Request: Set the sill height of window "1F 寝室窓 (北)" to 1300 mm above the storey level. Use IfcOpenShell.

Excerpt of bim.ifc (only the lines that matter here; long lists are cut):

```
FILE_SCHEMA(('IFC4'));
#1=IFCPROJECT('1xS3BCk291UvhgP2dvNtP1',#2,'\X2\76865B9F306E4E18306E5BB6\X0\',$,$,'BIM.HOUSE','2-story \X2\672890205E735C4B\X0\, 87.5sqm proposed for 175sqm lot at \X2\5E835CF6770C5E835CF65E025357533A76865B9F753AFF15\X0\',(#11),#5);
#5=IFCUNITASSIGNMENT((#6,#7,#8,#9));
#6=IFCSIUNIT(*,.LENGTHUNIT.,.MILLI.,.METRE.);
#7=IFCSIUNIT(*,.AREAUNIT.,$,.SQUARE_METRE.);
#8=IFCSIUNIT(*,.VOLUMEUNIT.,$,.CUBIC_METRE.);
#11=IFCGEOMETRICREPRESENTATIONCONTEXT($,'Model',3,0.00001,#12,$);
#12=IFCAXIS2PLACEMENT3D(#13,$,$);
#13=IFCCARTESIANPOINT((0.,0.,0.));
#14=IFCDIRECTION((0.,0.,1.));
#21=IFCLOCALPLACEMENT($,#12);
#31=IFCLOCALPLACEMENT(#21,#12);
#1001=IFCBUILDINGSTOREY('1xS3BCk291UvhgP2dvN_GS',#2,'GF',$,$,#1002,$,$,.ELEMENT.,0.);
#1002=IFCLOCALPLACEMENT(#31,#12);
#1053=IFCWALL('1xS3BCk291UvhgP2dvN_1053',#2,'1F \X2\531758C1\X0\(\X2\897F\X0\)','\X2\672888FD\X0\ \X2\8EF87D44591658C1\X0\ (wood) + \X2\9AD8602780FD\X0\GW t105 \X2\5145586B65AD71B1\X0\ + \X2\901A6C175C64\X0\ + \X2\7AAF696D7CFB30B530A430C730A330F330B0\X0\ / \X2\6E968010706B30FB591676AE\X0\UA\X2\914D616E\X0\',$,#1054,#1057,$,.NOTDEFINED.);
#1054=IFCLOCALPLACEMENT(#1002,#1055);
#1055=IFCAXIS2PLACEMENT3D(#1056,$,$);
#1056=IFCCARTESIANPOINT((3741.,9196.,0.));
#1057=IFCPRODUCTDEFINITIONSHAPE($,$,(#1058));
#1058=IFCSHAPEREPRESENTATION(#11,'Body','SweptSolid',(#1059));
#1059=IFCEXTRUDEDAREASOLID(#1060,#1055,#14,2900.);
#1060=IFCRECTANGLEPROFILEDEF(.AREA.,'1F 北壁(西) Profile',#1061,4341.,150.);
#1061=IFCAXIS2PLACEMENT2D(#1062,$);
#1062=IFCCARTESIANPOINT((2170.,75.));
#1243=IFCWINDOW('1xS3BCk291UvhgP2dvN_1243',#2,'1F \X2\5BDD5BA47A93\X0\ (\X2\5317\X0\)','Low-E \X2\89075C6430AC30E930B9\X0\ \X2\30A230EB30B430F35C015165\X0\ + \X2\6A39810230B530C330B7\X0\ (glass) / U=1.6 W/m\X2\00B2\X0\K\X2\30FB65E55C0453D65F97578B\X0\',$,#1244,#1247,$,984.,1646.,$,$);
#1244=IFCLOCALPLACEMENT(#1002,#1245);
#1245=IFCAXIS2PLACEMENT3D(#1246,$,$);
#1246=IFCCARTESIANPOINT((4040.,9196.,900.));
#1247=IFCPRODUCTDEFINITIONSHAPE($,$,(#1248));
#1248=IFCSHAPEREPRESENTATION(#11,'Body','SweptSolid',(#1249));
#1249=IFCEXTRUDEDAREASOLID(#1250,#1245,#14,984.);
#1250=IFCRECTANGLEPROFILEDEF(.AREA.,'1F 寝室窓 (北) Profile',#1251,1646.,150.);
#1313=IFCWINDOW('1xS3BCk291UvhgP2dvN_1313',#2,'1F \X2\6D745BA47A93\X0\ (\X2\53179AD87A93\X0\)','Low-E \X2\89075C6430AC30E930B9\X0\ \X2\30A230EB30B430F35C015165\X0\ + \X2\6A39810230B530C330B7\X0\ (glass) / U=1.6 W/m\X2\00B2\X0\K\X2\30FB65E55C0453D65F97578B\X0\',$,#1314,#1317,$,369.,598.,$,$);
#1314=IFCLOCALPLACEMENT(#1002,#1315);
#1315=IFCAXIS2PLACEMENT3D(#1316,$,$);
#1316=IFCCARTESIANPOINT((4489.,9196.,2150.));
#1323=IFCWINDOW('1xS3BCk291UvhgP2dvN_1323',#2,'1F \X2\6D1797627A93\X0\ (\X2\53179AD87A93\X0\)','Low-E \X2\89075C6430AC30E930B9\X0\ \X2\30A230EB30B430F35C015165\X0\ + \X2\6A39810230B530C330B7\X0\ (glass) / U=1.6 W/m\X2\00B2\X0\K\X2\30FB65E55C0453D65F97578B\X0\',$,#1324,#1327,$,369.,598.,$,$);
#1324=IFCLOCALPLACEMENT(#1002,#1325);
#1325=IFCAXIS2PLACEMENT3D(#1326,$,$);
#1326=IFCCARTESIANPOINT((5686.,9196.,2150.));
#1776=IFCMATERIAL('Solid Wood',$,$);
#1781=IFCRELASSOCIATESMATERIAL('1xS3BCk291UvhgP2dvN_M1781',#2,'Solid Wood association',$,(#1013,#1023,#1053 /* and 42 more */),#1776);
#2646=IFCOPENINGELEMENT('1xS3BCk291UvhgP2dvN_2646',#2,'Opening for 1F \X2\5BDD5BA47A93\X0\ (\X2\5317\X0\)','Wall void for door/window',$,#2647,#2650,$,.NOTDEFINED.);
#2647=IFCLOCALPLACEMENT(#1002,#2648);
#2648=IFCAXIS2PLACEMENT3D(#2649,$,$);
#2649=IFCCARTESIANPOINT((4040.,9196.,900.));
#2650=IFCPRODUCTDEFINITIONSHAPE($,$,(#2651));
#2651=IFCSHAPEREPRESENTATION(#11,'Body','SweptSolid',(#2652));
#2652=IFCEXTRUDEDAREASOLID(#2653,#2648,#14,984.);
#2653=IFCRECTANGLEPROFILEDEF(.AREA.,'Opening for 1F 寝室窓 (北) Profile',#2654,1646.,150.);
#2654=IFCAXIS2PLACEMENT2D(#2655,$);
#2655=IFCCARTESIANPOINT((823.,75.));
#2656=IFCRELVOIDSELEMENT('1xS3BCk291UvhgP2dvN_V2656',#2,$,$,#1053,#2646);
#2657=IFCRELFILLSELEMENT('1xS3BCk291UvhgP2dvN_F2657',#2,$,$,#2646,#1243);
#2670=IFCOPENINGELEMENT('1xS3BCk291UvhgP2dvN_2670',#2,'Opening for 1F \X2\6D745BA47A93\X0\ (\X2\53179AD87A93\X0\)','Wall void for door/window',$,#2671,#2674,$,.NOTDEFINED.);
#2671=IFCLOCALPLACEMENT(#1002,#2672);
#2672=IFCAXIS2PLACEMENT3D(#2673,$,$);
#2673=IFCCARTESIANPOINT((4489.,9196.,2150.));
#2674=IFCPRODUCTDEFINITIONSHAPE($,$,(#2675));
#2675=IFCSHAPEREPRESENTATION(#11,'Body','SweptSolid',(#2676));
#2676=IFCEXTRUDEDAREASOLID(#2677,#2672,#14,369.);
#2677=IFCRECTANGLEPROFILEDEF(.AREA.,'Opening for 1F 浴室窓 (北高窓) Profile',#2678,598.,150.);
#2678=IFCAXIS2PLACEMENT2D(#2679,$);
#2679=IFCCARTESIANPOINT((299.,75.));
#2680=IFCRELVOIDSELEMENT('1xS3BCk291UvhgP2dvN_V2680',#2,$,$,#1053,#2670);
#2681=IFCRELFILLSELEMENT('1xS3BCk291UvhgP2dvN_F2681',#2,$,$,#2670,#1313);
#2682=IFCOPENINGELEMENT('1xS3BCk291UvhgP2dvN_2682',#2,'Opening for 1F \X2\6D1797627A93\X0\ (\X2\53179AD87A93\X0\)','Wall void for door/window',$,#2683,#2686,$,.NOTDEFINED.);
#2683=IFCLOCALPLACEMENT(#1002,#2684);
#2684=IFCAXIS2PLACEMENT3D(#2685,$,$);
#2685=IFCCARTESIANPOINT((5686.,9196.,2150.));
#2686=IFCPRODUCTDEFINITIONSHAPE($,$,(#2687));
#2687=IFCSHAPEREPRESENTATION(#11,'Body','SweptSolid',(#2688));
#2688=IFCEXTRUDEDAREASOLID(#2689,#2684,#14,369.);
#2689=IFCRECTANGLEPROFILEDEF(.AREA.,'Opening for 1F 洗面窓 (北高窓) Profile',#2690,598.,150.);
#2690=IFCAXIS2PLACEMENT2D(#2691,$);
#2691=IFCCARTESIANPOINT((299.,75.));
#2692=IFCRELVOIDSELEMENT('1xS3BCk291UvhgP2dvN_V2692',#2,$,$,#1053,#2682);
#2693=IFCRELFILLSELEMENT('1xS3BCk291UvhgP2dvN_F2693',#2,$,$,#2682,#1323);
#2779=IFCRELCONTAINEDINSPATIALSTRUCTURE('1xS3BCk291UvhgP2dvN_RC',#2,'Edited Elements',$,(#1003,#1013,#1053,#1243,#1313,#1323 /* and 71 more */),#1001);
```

```python
import numpy as np
import ifcopenshell
import ifcopenshell.api.geometry
import ifcopenshell.geom
import ifcopenshell.util.element
import ifcopenshell.util.placement
import ifcopenshell.util.shape
import ifcopenshell.util.unit

model = ifcopenshell.open("bim.ifc")
unit_scale = ifcopenshell.util.unit.calculate_unit_scale(model)

window = model.by_guid("1xS3BCk291UvhgP2dvN_1243")
opening = window.FillsVoids[0].RelatingOpeningElement
storey = ifcopenshell.util.element.get_container(window, ifc_class="IfcBuildingStorey")
level = ifcopenshell.util.placement.get_local_placement(storey.ObjectPlacement)[2, 3]

# The opening's origin need not be at the sill, so measure its lowest point.
shape = ifcopenshell.geom.create_shape(ifcopenshell.geom.settings(), opening)
bottom = ifcopenshell.util.shape.get_shape_bottom_elevation(shape, shape.geometry) / unit_scale
dz = level + 1.3 / unit_scale - bottom

shift = np.array([0.0, 0.0, dz])
# The window is not placed relative to its opening, so move both.
for product in (opening, window):
    matrix = ifcopenshell.util.placement.get_local_placement(product.ObjectPlacement)
    matrix[:3, 3] += shift
    ifcopenshell.api.geometry.edit_object_placement(model, product=product, matrix=matrix, is_si=False)

print(f"moved by {dz * unit_scale:+.3f} m")

model.write("bim_updated.ifc")
```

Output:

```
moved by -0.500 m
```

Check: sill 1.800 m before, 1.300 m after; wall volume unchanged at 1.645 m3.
